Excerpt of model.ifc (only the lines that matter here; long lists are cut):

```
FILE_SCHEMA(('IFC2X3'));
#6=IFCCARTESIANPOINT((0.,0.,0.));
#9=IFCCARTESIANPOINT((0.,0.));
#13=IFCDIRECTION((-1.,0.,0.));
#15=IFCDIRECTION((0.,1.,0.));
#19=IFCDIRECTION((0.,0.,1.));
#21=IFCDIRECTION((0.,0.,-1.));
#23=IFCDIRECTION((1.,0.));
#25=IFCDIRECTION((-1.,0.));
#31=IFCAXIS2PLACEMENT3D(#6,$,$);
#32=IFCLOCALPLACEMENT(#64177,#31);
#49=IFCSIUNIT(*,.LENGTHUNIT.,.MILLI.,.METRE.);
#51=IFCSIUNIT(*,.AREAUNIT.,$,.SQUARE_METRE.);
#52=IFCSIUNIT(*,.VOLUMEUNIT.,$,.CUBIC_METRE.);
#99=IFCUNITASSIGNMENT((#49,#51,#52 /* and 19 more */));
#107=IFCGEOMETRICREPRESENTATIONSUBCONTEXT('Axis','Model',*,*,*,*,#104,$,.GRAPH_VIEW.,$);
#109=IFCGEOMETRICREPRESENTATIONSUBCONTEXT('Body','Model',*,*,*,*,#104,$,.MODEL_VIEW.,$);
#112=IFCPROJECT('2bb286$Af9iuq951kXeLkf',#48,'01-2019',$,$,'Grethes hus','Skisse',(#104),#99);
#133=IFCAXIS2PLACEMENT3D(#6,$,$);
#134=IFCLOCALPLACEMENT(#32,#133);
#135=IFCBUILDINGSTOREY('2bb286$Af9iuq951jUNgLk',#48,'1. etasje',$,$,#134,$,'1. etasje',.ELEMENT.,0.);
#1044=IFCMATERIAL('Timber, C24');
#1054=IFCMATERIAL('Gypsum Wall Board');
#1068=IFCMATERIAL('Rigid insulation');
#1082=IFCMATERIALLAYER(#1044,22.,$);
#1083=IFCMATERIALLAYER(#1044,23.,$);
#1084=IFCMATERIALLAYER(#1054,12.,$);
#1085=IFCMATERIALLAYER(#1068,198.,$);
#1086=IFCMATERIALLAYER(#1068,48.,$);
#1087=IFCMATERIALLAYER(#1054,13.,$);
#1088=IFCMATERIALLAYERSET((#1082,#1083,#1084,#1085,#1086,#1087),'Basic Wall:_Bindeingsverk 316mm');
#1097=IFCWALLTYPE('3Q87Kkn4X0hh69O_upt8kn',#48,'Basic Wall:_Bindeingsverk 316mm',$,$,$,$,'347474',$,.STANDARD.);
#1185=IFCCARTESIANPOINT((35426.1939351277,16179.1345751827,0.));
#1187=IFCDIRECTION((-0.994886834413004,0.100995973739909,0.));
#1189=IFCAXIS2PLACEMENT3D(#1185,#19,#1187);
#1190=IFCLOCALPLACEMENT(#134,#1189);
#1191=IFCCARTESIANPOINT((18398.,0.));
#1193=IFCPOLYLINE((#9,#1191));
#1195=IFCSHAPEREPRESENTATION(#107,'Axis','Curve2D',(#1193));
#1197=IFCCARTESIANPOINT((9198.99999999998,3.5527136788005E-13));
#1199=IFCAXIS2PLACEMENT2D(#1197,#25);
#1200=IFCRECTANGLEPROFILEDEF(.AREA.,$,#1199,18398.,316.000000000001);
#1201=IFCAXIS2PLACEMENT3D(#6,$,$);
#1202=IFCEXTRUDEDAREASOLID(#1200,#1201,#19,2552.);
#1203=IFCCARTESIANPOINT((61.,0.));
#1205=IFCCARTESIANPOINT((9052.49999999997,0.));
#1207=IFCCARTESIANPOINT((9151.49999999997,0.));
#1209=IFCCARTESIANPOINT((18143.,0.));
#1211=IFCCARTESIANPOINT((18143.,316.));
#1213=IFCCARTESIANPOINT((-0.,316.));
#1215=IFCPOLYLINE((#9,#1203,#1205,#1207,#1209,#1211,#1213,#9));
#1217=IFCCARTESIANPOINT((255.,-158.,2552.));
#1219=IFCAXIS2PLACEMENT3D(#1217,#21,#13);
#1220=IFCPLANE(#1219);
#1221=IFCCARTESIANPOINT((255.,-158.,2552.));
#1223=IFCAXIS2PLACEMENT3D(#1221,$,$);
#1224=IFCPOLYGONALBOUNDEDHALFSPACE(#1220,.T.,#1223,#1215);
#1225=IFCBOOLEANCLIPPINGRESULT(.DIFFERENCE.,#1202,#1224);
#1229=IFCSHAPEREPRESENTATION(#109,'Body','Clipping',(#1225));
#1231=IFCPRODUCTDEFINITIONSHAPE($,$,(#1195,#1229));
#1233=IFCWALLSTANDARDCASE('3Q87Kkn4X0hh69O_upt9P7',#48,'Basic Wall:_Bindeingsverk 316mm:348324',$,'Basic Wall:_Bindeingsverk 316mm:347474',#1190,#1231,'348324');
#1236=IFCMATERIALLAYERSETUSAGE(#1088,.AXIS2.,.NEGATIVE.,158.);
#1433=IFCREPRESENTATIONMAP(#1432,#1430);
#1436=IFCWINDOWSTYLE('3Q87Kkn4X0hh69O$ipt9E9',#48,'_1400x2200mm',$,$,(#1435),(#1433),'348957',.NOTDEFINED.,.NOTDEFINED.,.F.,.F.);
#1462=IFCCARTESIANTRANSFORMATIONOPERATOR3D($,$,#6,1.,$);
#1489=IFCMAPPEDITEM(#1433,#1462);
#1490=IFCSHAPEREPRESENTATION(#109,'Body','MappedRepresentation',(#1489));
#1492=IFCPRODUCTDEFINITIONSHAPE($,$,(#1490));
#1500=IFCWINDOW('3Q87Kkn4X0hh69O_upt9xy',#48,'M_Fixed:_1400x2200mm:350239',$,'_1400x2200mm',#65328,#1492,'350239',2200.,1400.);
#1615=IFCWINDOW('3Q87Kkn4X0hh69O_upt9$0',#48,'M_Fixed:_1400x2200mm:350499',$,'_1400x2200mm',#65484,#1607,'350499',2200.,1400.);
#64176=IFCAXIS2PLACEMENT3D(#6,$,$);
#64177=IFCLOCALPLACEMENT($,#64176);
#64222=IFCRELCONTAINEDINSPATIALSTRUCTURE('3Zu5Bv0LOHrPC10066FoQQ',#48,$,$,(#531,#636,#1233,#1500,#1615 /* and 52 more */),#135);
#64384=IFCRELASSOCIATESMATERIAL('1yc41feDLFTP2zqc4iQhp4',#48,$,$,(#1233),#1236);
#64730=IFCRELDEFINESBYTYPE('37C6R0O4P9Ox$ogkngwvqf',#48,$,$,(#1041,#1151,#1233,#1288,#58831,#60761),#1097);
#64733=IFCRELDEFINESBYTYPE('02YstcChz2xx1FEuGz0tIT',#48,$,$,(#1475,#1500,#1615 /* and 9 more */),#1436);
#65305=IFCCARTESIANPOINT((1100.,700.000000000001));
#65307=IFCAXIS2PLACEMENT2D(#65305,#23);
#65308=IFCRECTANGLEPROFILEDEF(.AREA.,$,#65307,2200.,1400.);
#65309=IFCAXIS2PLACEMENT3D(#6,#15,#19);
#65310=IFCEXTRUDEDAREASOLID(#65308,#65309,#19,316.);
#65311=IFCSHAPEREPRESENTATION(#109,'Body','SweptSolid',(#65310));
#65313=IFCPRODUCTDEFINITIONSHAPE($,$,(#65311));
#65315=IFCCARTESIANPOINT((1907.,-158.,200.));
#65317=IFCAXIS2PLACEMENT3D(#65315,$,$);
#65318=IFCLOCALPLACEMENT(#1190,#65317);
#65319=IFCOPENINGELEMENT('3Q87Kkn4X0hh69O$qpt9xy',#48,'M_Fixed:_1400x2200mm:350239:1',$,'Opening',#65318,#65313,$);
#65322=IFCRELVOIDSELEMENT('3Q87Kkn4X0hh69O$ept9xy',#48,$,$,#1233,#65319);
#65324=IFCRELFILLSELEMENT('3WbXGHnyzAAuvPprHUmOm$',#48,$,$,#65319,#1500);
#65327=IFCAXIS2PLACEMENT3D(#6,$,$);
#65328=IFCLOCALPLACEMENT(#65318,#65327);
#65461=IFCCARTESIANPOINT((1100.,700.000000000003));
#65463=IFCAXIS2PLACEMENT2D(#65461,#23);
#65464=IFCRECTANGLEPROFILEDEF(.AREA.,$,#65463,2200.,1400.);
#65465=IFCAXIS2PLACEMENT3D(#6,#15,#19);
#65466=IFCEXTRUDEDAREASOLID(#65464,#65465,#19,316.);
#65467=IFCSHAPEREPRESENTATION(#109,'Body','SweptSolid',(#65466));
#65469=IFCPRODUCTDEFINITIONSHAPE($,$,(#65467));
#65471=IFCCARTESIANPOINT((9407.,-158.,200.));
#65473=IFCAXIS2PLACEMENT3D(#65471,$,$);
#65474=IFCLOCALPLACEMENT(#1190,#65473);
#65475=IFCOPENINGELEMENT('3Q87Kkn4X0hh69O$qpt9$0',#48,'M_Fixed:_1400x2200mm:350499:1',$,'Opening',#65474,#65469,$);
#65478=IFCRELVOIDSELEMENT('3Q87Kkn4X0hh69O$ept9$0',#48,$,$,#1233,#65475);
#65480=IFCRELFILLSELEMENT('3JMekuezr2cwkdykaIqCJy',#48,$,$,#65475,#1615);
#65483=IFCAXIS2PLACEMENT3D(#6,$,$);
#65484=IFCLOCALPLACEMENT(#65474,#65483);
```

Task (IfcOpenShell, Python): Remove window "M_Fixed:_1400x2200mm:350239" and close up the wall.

```python
import ifcopenshell
import ifcopenshell.api.feature
import ifcopenshell.api.root
import ifcopenshell.geom
import ifcopenshell.util.shape

model = ifcopenshell.open("model.ifc")
settings = ifcopenshell.geom.settings()


def volume(element):
    """Net volume in cubic metres, openings subtracted."""
    shape = ifcopenshell.geom.create_shape(settings, element)
    return ifcopenshell.util.shape.get_volume(shape.geometry)


window = model.by_guid("3Q87Kkn4X0hh69O_upt9xy")
opening = window.FillsVoids[0].RelatingOpeningElement
wall = opening.VoidsElements[0].RelatingBuildingElement
before = volume(wall)

ifcopenshell.api.root.remove_product(model, product=window)
ifcopenshell.api.feature.remove_feature(model, feature=opening)

after = volume(wall)

print(f"wall volume {before:.3f} -> {after:.3f} m3")

model.write("model_edited.ifc")
```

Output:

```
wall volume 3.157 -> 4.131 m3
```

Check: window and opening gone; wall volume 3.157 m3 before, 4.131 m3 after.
